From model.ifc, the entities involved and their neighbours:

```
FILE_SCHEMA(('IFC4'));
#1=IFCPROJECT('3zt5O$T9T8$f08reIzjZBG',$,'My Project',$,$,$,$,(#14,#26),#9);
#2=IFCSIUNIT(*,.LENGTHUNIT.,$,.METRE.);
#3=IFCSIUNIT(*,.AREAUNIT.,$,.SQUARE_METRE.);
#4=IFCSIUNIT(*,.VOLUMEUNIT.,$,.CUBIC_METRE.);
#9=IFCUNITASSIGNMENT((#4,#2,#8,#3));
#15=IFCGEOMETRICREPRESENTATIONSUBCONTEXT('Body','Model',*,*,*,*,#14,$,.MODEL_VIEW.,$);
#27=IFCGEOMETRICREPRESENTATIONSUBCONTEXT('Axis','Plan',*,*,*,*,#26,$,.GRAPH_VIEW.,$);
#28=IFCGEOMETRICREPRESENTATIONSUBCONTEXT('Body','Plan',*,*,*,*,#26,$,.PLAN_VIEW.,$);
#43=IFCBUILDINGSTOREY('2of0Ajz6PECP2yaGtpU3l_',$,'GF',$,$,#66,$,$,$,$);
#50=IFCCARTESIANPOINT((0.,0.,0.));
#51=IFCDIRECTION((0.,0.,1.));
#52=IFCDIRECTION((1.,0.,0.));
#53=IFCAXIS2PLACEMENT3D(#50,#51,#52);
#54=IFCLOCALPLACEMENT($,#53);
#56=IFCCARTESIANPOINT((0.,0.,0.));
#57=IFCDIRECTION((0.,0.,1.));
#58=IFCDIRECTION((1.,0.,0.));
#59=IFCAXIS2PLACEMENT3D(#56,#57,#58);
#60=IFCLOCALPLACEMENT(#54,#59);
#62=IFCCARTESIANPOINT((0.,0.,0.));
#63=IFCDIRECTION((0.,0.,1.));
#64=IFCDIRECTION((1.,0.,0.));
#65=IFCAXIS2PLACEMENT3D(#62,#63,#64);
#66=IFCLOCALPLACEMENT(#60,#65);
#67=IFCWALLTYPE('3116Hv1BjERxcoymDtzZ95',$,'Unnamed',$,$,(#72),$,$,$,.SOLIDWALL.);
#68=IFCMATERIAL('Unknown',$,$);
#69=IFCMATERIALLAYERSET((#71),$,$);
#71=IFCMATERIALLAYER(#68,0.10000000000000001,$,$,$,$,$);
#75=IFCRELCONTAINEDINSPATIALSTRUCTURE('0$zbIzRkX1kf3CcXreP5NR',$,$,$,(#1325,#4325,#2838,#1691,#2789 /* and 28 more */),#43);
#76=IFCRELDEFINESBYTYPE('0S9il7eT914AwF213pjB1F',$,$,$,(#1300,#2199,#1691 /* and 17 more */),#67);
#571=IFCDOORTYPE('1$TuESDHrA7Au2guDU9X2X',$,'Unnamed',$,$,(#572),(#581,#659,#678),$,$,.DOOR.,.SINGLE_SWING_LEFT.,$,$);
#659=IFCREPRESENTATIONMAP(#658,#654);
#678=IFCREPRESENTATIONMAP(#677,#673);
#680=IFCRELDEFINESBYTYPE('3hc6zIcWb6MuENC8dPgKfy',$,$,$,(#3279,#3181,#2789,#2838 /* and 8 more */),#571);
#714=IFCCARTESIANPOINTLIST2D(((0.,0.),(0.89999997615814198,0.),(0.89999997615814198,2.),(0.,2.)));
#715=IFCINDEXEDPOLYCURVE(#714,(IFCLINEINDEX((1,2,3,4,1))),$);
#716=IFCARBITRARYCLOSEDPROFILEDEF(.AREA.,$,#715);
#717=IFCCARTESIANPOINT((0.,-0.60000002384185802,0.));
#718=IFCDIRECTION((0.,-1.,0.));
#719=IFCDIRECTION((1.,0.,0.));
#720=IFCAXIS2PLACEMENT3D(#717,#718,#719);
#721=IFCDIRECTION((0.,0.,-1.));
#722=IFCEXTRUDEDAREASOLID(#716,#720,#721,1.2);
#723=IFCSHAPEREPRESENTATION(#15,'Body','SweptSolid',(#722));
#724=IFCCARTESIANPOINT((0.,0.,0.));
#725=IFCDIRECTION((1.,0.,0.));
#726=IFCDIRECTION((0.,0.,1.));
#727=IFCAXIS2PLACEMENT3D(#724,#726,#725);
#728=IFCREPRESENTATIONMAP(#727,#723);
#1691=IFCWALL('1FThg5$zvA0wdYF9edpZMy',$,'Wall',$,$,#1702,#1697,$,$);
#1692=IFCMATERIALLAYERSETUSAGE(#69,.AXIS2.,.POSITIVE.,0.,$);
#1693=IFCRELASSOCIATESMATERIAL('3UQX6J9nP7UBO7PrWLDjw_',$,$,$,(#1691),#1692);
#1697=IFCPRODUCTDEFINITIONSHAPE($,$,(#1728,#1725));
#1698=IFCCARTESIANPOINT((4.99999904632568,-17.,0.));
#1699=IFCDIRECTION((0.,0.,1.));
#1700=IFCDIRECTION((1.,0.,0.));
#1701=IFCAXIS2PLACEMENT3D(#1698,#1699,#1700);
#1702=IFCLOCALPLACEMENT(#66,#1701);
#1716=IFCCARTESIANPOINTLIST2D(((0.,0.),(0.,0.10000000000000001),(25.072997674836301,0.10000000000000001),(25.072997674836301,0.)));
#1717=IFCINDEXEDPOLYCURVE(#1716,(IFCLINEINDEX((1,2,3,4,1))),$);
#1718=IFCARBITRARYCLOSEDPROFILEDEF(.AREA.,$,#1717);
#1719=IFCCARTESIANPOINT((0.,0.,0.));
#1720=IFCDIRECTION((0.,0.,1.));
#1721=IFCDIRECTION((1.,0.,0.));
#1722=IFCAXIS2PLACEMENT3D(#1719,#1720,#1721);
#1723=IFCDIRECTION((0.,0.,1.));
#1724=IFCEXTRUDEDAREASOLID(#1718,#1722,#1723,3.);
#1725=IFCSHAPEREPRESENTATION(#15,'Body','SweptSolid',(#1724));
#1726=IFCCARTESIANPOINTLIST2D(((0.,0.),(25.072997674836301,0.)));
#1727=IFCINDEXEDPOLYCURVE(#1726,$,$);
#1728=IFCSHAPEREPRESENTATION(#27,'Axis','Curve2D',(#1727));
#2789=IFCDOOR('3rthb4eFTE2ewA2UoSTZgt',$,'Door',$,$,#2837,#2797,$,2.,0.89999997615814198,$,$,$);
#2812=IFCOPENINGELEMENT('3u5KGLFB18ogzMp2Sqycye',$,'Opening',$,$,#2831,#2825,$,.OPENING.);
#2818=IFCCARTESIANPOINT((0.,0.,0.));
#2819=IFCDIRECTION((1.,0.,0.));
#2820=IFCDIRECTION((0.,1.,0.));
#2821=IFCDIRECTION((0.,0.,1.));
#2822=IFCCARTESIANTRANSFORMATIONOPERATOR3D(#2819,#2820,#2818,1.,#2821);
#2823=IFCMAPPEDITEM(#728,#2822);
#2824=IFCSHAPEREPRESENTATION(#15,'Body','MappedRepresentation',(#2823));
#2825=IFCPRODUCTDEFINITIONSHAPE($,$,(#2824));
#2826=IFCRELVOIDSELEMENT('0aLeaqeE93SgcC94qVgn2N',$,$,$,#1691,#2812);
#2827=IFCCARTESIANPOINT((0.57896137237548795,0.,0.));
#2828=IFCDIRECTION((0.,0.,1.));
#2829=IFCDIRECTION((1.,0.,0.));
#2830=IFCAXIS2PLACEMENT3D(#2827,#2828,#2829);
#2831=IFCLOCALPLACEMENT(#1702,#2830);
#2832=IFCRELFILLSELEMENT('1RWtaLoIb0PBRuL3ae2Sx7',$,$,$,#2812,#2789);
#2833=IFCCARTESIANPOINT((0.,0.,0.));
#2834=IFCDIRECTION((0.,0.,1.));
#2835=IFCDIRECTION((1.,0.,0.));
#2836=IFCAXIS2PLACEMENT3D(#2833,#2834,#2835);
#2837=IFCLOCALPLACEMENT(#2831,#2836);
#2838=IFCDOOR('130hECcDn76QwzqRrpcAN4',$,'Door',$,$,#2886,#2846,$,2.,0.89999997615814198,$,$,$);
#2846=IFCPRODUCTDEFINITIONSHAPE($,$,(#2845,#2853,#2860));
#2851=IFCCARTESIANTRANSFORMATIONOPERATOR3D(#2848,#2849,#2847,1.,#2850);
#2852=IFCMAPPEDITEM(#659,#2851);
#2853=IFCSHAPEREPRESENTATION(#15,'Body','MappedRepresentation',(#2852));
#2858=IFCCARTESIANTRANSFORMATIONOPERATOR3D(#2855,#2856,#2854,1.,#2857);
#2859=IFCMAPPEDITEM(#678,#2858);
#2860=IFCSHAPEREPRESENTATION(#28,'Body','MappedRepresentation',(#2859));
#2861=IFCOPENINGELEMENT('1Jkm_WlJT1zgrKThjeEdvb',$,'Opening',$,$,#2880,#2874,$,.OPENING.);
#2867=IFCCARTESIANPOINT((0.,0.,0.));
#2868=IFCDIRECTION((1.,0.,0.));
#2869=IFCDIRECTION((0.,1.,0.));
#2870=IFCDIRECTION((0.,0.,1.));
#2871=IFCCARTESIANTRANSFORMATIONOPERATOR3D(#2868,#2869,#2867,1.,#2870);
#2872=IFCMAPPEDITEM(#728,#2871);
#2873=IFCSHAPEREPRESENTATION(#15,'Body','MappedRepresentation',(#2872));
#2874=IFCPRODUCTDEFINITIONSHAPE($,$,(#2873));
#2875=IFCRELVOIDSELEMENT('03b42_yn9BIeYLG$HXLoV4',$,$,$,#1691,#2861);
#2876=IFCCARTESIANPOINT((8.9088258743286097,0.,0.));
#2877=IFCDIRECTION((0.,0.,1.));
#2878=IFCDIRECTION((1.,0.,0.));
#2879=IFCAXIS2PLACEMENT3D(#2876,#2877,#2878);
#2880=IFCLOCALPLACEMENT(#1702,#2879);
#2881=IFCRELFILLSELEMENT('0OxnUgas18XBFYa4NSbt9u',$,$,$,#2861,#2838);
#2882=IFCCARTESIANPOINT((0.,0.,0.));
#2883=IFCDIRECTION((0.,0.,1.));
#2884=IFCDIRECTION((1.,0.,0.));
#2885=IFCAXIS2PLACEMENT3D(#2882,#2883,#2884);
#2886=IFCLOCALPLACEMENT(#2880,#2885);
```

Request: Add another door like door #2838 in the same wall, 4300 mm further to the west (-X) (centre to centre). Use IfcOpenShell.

```python
import ifcopenshell
import ifcopenshell.api.feature
import ifcopenshell.api.geometry
import ifcopenshell.api.root
import ifcopenshell.geom
import ifcopenshell.util.element
import ifcopenshell.util.placement
import ifcopenshell.util.shape

model = ifcopenshell.open("model.ifc")
settings = ifcopenshell.geom.settings()


def volume(element):
    """Net volume in cubic metres, openings subtracted."""
    shape = ifcopenshell.geom.create_shape(settings, element)
    return ifcopenshell.util.shape.get_volume(shape.geometry)


door = model.by_guid("130hECcDn76QwzqRrpcAN4")
opening = door.FillsVoids[0].RelatingOpeningElement
wall = opening.VoidsElements[0].RelatingBuildingElement
before = volume(wall)
shift = ifcopenshell.util.placement.get_local_placement(wall.ObjectPlacement)[:3, 0] * -4.3

# copy_class copies the void relationship, type, container and properties, but no geometry.
new_opening = ifcopenshell.api.root.copy_class(model, product=opening)
new_opening.Representation = ifcopenshell.util.element.copy_deep(
    model, opening.Representation, exclude=["IfcGeometricRepresentationContext", "IfcRepresentationMap"]
)
new_door = ifcopenshell.api.root.copy_class(model, product=door)
new_door.Representation = ifcopenshell.util.element.copy_deep(
    model, door.Representation, exclude=["IfcGeometricRepresentationContext", "IfcRepresentationMap"]
)
ifcopenshell.api.feature.add_filling(model, opening=new_opening, element=new_door)

for old, new in ((opening, new_opening), (door, new_door)):
    matrix = ifcopenshell.util.placement.get_local_placement(old.ObjectPlacement)
    matrix[:3, 3] += shift
    ifcopenshell.api.geometry.edit_object_placement(model, product=new, matrix=matrix, is_si=False)

after = volume(wall)

print(f"wall volume {before:.3f} -> {after:.3f} m3")

model.write("model_rev.ifc")
```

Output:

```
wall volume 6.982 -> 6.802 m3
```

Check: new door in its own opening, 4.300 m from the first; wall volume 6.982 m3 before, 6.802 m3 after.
